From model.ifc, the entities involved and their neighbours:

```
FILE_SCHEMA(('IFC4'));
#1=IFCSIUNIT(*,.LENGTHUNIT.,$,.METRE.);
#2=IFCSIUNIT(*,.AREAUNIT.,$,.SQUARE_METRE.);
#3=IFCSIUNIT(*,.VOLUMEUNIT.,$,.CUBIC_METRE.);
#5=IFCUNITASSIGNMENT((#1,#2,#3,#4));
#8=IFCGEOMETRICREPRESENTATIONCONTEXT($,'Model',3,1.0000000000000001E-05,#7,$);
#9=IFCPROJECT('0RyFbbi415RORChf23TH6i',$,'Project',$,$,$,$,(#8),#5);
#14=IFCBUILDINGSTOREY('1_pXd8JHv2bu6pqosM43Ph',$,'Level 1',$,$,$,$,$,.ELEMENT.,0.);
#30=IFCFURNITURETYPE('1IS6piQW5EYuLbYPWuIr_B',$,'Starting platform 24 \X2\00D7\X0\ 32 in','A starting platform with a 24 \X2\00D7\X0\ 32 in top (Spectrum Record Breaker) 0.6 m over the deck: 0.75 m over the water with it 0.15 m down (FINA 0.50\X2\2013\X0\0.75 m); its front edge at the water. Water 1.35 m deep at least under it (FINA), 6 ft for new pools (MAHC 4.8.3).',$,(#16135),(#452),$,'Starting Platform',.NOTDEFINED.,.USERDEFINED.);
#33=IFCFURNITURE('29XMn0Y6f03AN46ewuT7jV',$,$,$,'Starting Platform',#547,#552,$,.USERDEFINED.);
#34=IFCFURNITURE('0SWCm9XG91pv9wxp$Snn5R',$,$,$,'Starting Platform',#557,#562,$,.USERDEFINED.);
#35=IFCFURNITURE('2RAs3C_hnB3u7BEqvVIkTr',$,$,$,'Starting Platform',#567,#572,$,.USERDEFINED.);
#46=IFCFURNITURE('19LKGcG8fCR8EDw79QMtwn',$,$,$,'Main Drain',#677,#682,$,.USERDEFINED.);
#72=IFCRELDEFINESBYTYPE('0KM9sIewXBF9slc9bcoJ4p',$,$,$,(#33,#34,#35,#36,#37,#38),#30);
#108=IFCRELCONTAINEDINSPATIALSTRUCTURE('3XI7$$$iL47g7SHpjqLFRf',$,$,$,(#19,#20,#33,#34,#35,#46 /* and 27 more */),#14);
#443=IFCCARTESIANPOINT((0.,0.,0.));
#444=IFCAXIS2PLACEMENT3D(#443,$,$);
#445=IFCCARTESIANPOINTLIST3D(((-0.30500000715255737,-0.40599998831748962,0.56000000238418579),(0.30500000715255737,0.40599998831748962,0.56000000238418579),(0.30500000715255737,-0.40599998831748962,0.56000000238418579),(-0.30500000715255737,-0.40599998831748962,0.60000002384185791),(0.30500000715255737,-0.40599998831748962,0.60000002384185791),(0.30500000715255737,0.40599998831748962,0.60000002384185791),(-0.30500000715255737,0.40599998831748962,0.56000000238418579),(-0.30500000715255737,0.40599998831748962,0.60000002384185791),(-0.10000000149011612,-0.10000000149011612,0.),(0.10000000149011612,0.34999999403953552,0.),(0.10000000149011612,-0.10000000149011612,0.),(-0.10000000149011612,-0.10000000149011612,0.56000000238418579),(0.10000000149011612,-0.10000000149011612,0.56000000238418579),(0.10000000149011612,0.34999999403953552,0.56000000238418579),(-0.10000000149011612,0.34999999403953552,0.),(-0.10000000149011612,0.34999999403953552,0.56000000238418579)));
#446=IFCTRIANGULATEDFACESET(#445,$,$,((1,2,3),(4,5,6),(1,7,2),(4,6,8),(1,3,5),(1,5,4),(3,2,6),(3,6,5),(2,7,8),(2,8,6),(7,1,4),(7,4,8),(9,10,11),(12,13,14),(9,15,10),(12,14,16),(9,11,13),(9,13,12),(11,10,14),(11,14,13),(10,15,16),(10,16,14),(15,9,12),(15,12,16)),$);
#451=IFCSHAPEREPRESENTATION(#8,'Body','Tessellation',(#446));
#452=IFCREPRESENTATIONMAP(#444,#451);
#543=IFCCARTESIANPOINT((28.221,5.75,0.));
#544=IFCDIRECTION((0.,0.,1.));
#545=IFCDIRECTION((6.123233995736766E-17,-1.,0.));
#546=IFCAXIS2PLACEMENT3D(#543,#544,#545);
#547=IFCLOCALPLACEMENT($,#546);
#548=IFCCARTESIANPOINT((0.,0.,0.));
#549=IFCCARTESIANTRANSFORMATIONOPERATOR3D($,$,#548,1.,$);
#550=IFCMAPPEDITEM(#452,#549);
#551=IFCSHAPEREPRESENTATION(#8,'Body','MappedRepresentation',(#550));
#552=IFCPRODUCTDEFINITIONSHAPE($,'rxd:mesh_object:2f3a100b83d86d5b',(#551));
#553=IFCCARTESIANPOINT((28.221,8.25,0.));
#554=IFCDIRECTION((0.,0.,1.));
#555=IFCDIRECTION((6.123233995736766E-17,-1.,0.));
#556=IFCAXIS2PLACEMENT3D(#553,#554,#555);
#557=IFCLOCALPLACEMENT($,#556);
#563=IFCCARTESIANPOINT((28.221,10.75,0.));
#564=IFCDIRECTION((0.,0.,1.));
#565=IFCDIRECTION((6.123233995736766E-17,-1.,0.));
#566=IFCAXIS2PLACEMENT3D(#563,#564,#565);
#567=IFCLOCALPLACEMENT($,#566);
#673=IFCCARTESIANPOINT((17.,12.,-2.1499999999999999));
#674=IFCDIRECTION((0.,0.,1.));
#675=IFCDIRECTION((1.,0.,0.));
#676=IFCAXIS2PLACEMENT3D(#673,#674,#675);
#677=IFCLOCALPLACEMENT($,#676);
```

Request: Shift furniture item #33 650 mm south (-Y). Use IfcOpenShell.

```python
import ifcopenshell
import ifcopenshell.api.geometry
import ifcopenshell.util.placement
import ifcopenshell.util.unit

model = ifcopenshell.open("model.ifc")
unit_scale = ifcopenshell.util.unit.calculate_unit_scale(model)

item = model.by_guid("29XMn0Y6f03AN46ewuT7jV")
matrix = ifcopenshell.util.placement.get_local_placement(item.ObjectPlacement)
matrix[1, 3] -= 0.65 / unit_scale
ifcopenshell.api.geometry.edit_object_placement(model, product=item, matrix=matrix, is_si=False)

print(ifcopenshell.util.placement.get_local_placement(item.ObjectPlacement).round(3) + 0.0)

model.write("model_v2.ifc")
```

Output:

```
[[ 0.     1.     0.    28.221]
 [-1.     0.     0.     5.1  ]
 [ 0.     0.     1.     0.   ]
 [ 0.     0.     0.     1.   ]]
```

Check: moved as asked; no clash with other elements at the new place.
